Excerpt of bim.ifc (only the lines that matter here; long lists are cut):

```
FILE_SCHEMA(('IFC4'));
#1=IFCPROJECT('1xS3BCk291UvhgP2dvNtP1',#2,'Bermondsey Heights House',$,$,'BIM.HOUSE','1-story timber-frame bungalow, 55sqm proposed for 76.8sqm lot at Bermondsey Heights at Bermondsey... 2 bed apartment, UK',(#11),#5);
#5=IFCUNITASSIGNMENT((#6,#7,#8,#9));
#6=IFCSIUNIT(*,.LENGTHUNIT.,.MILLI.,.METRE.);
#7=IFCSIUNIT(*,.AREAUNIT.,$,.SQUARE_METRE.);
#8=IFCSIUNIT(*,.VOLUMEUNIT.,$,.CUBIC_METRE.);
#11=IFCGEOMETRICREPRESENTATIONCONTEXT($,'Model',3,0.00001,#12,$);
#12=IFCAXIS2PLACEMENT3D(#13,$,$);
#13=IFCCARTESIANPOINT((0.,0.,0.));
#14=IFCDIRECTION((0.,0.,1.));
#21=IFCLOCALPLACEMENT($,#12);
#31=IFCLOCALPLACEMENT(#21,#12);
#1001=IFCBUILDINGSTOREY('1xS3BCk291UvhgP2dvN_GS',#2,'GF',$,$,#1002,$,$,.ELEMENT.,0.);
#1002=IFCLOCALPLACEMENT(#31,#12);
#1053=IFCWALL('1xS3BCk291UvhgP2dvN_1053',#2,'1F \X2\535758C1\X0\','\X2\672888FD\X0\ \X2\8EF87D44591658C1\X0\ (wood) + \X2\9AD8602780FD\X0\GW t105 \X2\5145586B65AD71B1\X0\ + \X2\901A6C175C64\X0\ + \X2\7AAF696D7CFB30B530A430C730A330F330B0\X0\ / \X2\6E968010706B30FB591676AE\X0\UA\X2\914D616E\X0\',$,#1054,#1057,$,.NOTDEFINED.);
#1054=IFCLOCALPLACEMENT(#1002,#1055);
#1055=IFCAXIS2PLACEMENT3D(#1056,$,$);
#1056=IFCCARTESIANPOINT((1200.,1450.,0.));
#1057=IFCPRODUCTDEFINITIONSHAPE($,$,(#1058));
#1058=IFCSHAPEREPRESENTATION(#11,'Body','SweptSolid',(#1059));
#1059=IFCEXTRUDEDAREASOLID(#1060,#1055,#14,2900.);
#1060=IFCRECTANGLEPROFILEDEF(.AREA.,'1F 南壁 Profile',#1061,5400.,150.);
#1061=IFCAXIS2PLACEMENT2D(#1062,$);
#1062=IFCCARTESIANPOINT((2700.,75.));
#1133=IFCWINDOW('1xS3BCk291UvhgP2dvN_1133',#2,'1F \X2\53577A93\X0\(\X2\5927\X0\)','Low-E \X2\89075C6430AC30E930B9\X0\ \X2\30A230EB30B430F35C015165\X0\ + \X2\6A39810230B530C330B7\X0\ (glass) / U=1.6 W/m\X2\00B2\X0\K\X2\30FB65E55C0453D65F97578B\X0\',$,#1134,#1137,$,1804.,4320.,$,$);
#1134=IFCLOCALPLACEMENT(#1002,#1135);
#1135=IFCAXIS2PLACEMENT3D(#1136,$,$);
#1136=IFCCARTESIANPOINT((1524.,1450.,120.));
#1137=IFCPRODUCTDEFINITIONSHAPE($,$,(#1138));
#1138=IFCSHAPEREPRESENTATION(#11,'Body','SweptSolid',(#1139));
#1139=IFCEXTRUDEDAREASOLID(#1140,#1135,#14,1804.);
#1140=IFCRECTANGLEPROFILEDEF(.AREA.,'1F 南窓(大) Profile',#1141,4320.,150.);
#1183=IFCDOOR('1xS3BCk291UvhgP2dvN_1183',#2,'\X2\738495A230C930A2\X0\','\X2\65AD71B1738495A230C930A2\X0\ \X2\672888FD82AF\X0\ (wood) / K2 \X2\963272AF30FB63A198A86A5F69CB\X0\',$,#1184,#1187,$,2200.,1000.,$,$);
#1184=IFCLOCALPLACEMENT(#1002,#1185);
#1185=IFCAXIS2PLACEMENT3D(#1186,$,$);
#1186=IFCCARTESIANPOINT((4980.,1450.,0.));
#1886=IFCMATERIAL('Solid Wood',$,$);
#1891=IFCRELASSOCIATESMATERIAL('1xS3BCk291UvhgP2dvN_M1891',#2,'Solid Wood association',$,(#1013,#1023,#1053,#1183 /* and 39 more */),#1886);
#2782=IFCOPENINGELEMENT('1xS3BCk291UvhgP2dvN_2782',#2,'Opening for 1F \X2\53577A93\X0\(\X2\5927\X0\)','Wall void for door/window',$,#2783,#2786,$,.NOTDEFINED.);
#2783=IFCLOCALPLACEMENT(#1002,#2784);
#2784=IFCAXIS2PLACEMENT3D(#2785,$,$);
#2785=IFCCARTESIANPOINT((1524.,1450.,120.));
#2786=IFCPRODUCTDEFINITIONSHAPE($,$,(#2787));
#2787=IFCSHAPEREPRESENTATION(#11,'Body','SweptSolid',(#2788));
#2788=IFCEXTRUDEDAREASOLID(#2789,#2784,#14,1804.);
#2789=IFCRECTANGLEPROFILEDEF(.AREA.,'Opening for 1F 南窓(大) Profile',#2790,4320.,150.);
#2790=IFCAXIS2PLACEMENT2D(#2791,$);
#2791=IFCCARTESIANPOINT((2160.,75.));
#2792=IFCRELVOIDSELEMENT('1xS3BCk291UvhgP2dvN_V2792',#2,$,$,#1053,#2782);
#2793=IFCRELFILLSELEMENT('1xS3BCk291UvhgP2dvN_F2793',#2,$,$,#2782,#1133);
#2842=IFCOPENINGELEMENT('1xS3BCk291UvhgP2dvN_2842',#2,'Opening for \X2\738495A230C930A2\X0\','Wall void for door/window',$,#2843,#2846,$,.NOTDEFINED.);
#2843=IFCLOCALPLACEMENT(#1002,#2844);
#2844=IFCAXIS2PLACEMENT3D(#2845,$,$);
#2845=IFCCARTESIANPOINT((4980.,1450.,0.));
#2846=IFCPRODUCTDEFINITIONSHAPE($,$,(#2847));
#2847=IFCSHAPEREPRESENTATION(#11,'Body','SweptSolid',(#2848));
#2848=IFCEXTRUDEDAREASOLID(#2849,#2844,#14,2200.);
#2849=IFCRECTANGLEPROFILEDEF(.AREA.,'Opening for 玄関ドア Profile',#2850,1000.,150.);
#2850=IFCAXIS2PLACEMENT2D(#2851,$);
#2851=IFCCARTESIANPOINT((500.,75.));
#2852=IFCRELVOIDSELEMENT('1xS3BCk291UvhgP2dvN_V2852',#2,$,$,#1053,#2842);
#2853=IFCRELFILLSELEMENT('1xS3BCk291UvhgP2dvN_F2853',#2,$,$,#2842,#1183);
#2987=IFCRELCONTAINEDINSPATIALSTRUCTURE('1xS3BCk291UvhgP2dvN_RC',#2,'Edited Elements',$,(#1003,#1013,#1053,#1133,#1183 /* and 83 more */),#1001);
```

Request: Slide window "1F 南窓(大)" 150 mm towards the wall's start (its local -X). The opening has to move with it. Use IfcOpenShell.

```python
import ifcopenshell
import ifcopenshell.api.geometry
import ifcopenshell.util.placement

model = ifcopenshell.open("bim.ifc")

window = model.by_guid("1xS3BCk291UvhgP2dvN_1133")
opening = window.FillsVoids[0].RelatingOpeningElement
wall = opening.VoidsElements[0].RelatingBuildingElement

wall_matrix = ifcopenshell.util.placement.get_local_placement(wall.ObjectPlacement)
shift = wall_matrix[:3, 0] * -150.0
before = ifcopenshell.util.placement.get_local_placement(window.ObjectPlacement)[:3, 3].copy()

# The window is not placed relative to its opening, so move both.
for product in (opening, window):
    matrix = ifcopenshell.util.placement.get_local_placement(product.ObjectPlacement)
    matrix[:3, 3] += shift
    ifcopenshell.api.geometry.edit_object_placement(model, product=product, matrix=matrix, is_si=False)

after = ifcopenshell.util.placement.get_local_placement(window.ObjectPlacement)[:3, 3]
print("window moved by", (after - before).round(3) + 0.0)

model.write("bim_edited.ifc")
```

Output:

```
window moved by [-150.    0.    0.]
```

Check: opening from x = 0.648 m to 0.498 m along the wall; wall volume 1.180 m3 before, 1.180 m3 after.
